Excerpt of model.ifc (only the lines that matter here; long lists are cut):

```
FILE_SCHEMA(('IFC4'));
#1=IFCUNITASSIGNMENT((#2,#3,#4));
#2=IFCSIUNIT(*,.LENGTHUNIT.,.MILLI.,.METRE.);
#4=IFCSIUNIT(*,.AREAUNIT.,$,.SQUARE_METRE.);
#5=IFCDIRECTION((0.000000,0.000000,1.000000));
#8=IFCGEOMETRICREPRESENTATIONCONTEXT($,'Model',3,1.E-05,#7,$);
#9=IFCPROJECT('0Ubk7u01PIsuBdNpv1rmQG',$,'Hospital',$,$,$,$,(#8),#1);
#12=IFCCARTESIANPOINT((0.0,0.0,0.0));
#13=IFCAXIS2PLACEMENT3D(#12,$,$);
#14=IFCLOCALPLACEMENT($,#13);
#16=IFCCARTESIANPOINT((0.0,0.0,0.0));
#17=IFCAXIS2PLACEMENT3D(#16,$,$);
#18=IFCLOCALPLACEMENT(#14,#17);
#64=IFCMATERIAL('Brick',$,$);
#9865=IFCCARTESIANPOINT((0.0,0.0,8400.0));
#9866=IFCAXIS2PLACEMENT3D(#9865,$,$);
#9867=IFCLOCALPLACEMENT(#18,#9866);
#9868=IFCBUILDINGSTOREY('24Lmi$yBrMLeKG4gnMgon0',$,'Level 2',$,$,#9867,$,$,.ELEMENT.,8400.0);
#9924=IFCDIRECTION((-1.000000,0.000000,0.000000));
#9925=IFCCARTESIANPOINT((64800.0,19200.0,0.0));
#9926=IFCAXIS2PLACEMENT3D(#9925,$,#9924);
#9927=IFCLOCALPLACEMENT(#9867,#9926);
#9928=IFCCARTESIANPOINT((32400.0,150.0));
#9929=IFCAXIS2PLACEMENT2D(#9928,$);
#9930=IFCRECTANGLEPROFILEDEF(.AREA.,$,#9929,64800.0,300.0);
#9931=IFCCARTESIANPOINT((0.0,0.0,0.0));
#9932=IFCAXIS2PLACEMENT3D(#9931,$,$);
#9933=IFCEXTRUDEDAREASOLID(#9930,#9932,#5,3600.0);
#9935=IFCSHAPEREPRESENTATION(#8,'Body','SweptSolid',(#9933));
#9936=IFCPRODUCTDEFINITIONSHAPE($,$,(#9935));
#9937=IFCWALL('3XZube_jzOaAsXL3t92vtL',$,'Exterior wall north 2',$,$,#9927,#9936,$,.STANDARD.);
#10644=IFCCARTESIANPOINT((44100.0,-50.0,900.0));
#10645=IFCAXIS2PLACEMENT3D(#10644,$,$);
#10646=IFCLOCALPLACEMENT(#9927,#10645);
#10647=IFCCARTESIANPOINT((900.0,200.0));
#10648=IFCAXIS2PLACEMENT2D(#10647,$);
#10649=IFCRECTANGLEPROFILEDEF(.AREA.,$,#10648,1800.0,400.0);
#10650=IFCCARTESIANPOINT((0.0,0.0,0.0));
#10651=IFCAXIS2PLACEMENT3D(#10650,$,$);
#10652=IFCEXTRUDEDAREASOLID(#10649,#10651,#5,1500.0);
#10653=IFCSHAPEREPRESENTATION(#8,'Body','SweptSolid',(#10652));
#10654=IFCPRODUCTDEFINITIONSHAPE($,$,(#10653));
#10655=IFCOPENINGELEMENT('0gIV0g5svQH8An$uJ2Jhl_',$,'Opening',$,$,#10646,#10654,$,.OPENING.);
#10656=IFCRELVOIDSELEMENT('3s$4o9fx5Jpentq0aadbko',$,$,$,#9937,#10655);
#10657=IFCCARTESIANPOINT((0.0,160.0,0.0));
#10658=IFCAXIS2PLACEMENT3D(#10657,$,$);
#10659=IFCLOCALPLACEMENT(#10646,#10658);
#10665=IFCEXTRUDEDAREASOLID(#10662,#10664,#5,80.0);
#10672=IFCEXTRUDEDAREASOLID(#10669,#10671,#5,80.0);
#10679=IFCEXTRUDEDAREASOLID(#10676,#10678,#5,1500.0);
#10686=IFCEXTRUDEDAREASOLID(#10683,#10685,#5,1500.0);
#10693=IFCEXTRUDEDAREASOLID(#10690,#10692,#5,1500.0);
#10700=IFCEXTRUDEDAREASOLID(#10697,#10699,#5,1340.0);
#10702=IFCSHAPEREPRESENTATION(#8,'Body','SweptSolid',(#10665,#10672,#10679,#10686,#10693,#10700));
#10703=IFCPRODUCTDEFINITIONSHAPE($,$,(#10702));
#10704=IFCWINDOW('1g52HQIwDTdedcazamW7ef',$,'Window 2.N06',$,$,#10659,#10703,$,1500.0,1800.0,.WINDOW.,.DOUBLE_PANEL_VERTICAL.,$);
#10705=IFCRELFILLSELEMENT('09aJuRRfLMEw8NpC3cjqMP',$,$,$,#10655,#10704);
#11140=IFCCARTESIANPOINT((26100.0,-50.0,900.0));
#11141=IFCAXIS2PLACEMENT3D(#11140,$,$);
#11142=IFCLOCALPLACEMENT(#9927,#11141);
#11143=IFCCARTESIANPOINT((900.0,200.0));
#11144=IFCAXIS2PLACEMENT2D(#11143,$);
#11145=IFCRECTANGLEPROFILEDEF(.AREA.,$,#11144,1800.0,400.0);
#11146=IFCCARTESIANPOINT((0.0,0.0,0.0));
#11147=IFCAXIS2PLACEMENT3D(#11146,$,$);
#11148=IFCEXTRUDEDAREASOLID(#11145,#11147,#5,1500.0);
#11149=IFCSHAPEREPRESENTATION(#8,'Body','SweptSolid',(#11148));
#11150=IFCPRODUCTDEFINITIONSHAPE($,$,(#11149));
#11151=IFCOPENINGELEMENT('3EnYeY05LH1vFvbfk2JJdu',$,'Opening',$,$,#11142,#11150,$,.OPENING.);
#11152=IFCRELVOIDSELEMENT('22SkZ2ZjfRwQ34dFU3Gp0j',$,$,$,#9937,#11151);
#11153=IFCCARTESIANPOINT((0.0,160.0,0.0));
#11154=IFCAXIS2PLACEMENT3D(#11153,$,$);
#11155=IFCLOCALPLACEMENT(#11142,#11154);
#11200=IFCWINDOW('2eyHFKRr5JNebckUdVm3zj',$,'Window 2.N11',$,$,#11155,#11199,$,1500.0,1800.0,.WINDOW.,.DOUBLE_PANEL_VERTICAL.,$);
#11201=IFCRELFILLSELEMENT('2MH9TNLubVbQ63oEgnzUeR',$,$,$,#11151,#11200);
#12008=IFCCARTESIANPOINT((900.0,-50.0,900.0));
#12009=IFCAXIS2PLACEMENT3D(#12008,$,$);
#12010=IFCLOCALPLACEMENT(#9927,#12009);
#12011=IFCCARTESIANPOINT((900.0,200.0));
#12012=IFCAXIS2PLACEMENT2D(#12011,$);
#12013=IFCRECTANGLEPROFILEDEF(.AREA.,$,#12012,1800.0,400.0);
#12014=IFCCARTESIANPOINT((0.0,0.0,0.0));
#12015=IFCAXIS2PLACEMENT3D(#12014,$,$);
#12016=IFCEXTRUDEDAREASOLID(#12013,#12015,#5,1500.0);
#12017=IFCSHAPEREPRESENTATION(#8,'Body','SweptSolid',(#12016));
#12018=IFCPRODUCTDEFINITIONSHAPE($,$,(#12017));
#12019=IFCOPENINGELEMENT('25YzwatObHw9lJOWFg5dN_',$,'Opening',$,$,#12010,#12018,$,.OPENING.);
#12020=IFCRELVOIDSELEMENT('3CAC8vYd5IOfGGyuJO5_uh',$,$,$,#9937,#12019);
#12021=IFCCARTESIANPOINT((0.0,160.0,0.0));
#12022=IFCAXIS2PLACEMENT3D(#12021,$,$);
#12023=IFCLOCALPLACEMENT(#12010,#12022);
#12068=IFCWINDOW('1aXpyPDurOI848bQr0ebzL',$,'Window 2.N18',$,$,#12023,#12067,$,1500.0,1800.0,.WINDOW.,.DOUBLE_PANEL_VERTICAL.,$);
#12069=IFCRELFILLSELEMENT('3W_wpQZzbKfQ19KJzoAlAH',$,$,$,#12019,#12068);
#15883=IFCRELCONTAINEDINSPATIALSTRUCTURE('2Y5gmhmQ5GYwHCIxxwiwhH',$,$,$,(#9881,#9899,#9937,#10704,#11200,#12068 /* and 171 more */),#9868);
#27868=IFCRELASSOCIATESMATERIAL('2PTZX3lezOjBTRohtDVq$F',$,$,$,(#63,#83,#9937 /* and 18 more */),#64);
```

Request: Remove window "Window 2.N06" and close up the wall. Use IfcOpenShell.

```python
import ifcopenshell
import ifcopenshell.api.feature
import ifcopenshell.api.root
import ifcopenshell.geom
import ifcopenshell.util.shape

model = ifcopenshell.open("model.ifc")
settings = ifcopenshell.geom.settings()


def volume(element):
    """Net volume in cubic metres, openings subtracted."""
    shape = ifcopenshell.geom.create_shape(settings, element)
    return ifcopenshell.util.shape.get_volume(shape.geometry)


window = model.by_id(10704)
opening = window.FillsVoids[0].RelatingOpeningElement
wall = opening.VoidsElements[0].RelatingBuildingElement
before = volume(wall)

ifcopenshell.api.root.remove_product(model, product=window)
ifcopenshell.api.feature.remove_feature(model, feature=opening)

after = volume(wall)

print(f"wall volume {before:.3f} -> {after:.3f} m3")

model.write("model_edited.ifc")
```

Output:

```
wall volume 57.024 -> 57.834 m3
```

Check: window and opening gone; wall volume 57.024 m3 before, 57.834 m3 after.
